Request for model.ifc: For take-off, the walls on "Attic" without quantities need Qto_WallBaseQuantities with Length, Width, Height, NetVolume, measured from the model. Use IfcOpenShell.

First a look at what the model holds.

```python
import ifcopenshell
import ifcopenshell.util.element
import ifcopenshell.util.unit

model = ifcopenshell.open("model.ifc")
print(model.schema)
for unit_type in ("LENGTHUNIT", "AREAUNIT", "VOLUMEUNIT"):
    print(unit_type, ifcopenshell.util.unit.calculate_unit_scale(model, unit_type))
storey = next(s for s in model.by_type("IfcBuildingStorey") if s.Name == "Attic")
walls = [e for e in ifcopenshell.util.element.get_decomposition(storey) if e.is_a("IfcWall")]
for e in sorted(walls, key=lambda e: e.id()):
    print(e.id(), e.is_a(), e.Name, list(ifcopenshell.util.element.get_psets(e, qtos_only=True)), sep=" | ")
```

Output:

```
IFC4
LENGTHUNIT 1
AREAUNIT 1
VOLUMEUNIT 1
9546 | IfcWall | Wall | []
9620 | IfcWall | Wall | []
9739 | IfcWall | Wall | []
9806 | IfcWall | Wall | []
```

```python
import ifcopenshell
import ifcopenshell.api.pset
import ifcopenshell.geom
import ifcopenshell.util.element
import ifcopenshell.util.shape
import ifcopenshell.util.unit

model = ifcopenshell.open("model.ifc")
unit_scale = ifcopenshell.util.unit.calculate_unit_scale(model)
volume_scale = ifcopenshell.util.unit.calculate_unit_scale(model, "VOLUMEUNIT")
settings = ifcopenshell.geom.settings()

storey = next(s for s in model.by_type("IfcBuildingStorey") if s.Name == "Attic")
walls = [e for e in ifcopenshell.util.element.get_decomposition(storey) if e.is_a("IfcWall")]

for e in sorted(walls, key=lambda e: e.id()):
    if ifcopenshell.util.element.get_psets(e, qtos_only=True, should_inherit=False):
        continue
    # Geometry comes back in metres, in the element's own axes.
    shape = ifcopenshell.geom.create_shape(settings, e)
    values = {
        "Length": ifcopenshell.util.shape.get_x(shape.geometry) / unit_scale,
        "Width": ifcopenshell.util.shape.get_y(shape.geometry) / unit_scale,
        "Height": ifcopenshell.util.shape.get_z(shape.geometry) / unit_scale,
        "NetVolume": ifcopenshell.util.shape.get_volume(shape.geometry) / volume_scale,
    }
    qto = ifcopenshell.api.pset.add_qto(model, product=e, name="Qto_WallBaseQuantities")
    ifcopenshell.api.pset.edit_qto(model, qto=qto, properties=values)
    print(e.id(), {k: round(v, 3) for k, v in values.items()})

model.write("model-out.ifc")
```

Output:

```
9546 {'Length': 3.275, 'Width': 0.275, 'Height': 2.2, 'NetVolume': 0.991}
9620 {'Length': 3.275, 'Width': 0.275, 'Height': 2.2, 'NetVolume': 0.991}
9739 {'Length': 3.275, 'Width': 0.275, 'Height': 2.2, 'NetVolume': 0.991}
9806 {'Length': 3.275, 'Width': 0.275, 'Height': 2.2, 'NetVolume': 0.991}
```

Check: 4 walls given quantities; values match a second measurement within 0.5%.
